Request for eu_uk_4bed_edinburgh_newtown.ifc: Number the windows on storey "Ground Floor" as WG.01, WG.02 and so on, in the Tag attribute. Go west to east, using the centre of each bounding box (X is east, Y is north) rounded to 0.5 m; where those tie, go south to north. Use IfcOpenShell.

First a look at what the model holds.

```python
import ifcopenshell
import ifcopenshell.util.element
import ifcopenshell.util.placement

model = ifcopenshell.open("eu_uk_4bed_edinburgh_newtown.ifc")
print(model.schema)
storey = next(s for s in model.by_type("IfcBuildingStorey") if s.Name == "Ground Floor")
windows = [e for e in ifcopenshell.util.element.get_decomposition(storey) if e.is_a("IfcWindow")]
for e in sorted(windows, key=lambda e: e.id()):
    origin = ifcopenshell.util.placement.get_local_placement(e.ObjectPlacement)[:3, 3]
    print(e.id(), e.Tag, e.Name, origin.round(2) + 0.0, sep=" | ")
```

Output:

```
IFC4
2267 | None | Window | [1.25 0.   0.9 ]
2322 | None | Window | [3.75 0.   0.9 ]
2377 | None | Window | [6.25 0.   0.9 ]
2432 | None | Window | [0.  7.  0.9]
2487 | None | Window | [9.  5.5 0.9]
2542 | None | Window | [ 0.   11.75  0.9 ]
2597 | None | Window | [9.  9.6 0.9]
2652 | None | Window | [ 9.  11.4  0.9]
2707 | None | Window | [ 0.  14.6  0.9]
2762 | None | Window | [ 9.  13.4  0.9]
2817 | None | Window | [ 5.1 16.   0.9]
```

```python
import ifcopenshell
import ifcopenshell.geom
import ifcopenshell.util.element
import ifcopenshell.util.shape

model = ifcopenshell.open("eu_uk_4bed_edinburgh_newtown.ifc")
settings = ifcopenshell.geom.settings()
settings.set("use-world-coords", True)


def centre(element):
    shape = ifcopenshell.geom.create_shape(settings, element)
    return ifcopenshell.util.shape.get_bbox_centroid(shape.geometry)


storey = next(s for s in model.by_type("IfcBuildingStorey") if s.Name == "Ground Floor")
windows = [e for e in ifcopenshell.util.element.get_decomposition(storey) if e.is_a("IfcWindow")]

# Insertion points can sit at a corner or the storey origin, so sort by the geometry (in metres).
centres = {e: centre(e) for e in windows}
windows.sort(key=lambda e: (round(centres[e][0] / 0.5), centres[e][1]))

for i, e in enumerate(windows, start=1):
    number = f"WG.{i:02d}"
    e.Tag = number
    print(e.id(), number)

model.write("eu_uk_4bed_edinburgh_newtown_v2.ifc")
```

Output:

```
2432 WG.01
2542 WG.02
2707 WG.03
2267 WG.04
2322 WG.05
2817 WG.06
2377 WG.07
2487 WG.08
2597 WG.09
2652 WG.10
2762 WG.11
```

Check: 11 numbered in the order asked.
